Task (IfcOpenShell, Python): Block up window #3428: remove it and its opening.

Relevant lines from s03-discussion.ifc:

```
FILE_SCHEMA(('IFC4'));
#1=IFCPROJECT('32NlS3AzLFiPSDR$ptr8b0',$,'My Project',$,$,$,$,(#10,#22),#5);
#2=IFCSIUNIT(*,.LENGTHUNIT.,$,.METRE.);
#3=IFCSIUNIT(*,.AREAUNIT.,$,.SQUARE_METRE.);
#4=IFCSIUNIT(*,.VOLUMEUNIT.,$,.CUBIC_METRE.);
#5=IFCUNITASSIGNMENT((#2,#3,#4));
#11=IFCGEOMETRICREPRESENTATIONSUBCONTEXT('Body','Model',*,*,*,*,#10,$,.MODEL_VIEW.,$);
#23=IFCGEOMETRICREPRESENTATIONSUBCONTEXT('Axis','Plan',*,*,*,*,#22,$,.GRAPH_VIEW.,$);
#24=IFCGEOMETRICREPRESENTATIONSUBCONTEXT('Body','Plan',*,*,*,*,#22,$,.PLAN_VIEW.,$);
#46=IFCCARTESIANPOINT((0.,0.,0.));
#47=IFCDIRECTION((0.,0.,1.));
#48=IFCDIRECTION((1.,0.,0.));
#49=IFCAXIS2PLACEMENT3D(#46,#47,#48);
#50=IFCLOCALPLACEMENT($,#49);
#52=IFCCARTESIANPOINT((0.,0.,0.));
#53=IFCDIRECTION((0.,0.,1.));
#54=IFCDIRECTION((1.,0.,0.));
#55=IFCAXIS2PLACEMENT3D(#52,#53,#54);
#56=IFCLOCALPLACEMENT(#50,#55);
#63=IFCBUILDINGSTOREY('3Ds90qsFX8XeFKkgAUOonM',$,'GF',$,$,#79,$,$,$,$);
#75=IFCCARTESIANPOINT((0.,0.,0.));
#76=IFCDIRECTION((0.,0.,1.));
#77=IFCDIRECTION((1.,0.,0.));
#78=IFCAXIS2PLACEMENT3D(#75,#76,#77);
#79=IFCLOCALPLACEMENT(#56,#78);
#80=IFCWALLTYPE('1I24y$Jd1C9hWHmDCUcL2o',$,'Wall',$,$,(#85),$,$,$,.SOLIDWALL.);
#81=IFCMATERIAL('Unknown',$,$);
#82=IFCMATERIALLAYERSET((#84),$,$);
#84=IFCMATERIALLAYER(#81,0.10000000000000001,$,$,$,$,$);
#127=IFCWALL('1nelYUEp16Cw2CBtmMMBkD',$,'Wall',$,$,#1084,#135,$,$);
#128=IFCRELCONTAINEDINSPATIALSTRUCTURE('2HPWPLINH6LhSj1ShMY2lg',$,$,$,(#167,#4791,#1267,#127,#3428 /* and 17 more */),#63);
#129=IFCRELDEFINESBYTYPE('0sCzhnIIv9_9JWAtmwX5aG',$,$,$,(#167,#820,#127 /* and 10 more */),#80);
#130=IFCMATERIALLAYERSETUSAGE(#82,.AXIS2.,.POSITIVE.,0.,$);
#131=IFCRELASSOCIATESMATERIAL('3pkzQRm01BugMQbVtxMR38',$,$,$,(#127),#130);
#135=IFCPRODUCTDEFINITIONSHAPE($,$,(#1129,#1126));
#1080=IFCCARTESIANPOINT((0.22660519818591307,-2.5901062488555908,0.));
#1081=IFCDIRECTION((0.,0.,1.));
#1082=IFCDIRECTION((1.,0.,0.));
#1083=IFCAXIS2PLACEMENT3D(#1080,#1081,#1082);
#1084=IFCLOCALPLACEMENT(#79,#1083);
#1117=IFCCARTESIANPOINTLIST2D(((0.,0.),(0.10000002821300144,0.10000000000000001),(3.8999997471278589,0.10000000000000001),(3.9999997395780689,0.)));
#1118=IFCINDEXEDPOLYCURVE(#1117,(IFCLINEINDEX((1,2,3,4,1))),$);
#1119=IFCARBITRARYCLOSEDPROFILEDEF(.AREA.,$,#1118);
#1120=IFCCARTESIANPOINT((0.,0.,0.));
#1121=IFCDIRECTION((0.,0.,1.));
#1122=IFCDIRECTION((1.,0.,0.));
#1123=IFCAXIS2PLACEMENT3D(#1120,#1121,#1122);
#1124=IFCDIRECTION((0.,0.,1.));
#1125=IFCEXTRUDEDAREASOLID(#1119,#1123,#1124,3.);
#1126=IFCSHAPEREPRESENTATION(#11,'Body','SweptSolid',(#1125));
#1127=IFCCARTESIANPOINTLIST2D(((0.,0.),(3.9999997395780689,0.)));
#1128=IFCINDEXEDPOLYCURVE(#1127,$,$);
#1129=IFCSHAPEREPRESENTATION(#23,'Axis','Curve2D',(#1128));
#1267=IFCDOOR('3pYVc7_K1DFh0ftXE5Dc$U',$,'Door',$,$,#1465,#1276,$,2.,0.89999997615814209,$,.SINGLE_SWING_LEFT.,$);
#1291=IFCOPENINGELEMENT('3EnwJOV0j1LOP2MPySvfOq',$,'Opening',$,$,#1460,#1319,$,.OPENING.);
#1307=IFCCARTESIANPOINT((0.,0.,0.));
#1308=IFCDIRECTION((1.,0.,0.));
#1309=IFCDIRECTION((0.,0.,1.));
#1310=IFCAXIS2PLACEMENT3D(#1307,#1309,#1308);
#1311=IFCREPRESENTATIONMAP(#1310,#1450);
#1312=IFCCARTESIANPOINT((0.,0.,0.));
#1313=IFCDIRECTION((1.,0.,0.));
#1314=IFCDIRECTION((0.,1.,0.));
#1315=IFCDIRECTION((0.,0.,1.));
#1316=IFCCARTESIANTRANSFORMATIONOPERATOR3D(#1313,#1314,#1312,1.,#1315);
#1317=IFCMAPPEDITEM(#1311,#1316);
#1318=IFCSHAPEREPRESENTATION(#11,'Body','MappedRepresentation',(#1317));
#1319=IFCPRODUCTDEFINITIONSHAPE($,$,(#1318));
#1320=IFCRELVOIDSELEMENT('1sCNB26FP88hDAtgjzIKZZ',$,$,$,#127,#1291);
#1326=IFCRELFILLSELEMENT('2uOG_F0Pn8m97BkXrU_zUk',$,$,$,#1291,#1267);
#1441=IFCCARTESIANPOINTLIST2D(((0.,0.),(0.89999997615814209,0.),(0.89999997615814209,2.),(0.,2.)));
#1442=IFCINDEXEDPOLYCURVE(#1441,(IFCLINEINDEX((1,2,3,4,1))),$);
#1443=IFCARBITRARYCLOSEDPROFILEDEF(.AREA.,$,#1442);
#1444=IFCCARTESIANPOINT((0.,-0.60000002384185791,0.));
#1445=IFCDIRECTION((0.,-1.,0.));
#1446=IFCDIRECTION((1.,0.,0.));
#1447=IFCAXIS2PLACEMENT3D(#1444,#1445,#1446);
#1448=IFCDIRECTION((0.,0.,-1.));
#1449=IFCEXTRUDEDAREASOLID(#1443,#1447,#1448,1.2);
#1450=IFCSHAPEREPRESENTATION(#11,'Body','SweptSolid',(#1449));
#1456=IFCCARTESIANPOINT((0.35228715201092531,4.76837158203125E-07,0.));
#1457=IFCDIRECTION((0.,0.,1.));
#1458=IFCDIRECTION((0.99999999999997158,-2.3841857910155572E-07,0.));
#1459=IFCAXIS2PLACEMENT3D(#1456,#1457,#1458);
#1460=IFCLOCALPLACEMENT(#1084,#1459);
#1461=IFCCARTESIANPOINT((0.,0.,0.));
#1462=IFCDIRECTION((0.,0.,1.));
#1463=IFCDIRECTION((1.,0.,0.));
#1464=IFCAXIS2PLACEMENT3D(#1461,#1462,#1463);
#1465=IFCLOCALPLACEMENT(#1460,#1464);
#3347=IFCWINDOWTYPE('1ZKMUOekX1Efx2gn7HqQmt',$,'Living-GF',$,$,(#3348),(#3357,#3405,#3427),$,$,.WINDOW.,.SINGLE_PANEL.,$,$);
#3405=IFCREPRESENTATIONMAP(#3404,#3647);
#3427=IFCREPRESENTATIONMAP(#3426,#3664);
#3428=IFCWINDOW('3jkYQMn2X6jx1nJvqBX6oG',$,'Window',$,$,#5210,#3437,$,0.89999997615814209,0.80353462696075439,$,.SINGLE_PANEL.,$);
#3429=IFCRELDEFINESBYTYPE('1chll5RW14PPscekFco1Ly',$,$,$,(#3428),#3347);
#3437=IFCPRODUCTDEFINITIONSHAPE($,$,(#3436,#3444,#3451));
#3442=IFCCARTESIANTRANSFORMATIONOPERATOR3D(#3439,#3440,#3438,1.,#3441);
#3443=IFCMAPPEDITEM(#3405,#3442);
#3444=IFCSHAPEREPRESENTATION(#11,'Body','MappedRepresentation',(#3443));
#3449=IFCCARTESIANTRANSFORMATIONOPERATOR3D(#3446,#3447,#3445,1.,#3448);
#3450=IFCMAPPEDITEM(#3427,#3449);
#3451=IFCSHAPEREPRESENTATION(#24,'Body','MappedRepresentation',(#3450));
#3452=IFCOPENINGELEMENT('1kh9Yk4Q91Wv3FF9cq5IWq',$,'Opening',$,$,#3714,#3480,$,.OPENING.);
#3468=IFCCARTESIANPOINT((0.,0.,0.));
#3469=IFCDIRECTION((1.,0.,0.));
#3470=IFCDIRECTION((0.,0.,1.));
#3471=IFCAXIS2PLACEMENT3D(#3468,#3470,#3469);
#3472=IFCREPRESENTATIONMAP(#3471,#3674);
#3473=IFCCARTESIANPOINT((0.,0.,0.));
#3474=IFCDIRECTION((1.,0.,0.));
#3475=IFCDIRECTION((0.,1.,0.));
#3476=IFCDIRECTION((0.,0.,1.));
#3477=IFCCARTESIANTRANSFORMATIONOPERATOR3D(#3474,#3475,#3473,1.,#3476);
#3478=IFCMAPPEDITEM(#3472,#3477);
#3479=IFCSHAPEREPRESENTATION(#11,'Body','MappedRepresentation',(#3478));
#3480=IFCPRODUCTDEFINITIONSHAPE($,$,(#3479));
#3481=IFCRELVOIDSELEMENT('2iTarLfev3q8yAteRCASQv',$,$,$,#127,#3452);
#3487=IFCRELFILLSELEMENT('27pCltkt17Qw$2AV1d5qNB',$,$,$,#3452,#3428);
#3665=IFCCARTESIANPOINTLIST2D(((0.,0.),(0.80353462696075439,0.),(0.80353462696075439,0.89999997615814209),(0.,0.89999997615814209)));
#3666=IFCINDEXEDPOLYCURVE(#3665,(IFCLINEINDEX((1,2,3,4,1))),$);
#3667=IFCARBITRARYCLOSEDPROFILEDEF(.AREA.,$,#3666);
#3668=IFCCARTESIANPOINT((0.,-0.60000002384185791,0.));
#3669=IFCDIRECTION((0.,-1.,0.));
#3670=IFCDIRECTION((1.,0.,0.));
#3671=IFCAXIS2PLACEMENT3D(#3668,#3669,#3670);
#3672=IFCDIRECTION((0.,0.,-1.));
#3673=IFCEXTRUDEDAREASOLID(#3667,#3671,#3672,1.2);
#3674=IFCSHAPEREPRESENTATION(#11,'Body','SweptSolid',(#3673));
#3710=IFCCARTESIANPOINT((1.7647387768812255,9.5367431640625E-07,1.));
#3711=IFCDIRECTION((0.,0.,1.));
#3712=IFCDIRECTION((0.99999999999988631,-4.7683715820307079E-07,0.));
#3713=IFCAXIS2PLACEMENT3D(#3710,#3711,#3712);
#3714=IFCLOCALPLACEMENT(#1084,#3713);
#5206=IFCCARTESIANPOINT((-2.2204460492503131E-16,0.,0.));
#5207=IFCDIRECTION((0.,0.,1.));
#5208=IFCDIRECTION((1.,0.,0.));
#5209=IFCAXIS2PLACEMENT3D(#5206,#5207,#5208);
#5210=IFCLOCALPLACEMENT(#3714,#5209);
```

```python
import ifcopenshell
import ifcopenshell.api.feature
import ifcopenshell.api.root
import ifcopenshell.geom
import ifcopenshell.util.shape

model = ifcopenshell.open("s03-discussion.ifc")
settings = ifcopenshell.geom.settings()


def volume(element):
    """Net volume in cubic metres, openings subtracted."""
    shape = ifcopenshell.geom.create_shape(settings, element)
    return ifcopenshell.util.shape.get_volume(shape.geometry)


window = model.by_guid("3jkYQMn2X6jx1nJvqBX6oG")
opening = window.FillsVoids[0].RelatingOpeningElement
wall = opening.VoidsElements[0].RelatingBuildingElement
before = volume(wall)

ifcopenshell.api.root.remove_product(model, product=window)
ifcopenshell.api.feature.remove_feature(model, feature=opening)

after = volume(wall)

print(f"wall volume {before:.3f} -> {after:.3f} m3")

model.write("s03-discussion_edited.ifc")
```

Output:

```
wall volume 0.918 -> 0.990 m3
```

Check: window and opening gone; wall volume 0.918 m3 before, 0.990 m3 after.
